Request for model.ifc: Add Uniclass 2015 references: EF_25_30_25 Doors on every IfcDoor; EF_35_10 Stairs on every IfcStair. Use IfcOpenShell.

First a look at what the model holds.

```python
import ifcopenshell

model = ifcopenshell.open("model.ifc")
print(model.schema)
print("classifications:", [c.Name for c in model.by_type("IfcClassification")])
for ifc_class in ("IfcDoor", "IfcRoof", "IfcStair", "IfcWall", "IfcWindow"):
    print(ifc_class, len(model.by_type(ifc_class)))
```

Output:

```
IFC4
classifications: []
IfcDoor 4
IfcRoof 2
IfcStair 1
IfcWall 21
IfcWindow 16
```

```python
import ifcopenshell
import ifcopenshell.api.classification

model = ifcopenshell.open("model.ifc")

system = ifcopenshell.api.classification.add_classification(model, classification="Uniclass 2015")

codes = {
    "IfcDoor": ("EF_25_30_25", "Doors"),
    "IfcStair": ("EF_35_10", "Stairs"),
}
for ifc_class, (code, name) in codes.items():
    products = model.by_type(ifc_class)
    ifcopenshell.api.classification.add_reference(
        model, products=products, classification=system, identification=code, name=name
    )
    print(code, len(products))

model.write("model_edited.ifc")
```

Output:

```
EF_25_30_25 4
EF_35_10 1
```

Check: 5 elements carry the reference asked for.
